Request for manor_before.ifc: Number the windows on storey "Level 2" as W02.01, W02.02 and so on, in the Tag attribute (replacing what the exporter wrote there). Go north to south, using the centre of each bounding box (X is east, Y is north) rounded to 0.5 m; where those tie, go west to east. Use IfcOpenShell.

First a look at what the model holds.

```python
import ifcopenshell
import ifcopenshell.util.element
import ifcopenshell.util.placement

model = ifcopenshell.open("manor_before.ifc")
print(model.schema)
storey = next(s for s in model.by_type("IfcBuildingStorey") if s.Name == "Level 2")
windows = [e for e in ifcopenshell.util.element.get_decomposition(storey) if e.is_a("IfcWindow")]
for e in sorted(windows, key=lambda e: e.id()):
    origin = ifcopenshell.util.placement.get_local_placement(e.ObjectPlacement)[:3, 3]
    print(e.id(), e.Tag, e.Name, origin.round(2) + 0.0, sep=" | ")
```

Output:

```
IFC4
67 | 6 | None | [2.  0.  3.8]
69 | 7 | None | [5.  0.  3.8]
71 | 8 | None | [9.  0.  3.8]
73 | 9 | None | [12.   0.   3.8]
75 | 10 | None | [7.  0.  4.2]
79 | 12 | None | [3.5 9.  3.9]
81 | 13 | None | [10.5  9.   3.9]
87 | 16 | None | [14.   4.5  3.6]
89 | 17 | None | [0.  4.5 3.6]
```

```python
import ifcopenshell
import ifcopenshell.geom
import ifcopenshell.util.element
import ifcopenshell.util.shape

model = ifcopenshell.open("manor_before.ifc")
settings = ifcopenshell.geom.settings()
settings.set("use-world-coords", True)


def centre(element):
    shape = ifcopenshell.geom.create_shape(settings, element)
    return ifcopenshell.util.shape.get_bbox_centroid(shape.geometry)


storey = next(s for s in model.by_type("IfcBuildingStorey") if s.Name == "Level 2")
windows = [e for e in ifcopenshell.util.element.get_decomposition(storey) if e.is_a("IfcWindow")]

# Insertion points can sit at a corner or the storey origin, so sort by the geometry (in metres).
centres = {e: centre(e) for e in windows}
windows.sort(key=lambda e: (-round(centres[e][1] / 0.5), centres[e][0]))

for i, e in enumerate(windows, start=1):
    number = f"W02.{i:02d}"
    e.Tag = number
    print(e.id(), number)

model.write("manor_before_v2.ifc")
```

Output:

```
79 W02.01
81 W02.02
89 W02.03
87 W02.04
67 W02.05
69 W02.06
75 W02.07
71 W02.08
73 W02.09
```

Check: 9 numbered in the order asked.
